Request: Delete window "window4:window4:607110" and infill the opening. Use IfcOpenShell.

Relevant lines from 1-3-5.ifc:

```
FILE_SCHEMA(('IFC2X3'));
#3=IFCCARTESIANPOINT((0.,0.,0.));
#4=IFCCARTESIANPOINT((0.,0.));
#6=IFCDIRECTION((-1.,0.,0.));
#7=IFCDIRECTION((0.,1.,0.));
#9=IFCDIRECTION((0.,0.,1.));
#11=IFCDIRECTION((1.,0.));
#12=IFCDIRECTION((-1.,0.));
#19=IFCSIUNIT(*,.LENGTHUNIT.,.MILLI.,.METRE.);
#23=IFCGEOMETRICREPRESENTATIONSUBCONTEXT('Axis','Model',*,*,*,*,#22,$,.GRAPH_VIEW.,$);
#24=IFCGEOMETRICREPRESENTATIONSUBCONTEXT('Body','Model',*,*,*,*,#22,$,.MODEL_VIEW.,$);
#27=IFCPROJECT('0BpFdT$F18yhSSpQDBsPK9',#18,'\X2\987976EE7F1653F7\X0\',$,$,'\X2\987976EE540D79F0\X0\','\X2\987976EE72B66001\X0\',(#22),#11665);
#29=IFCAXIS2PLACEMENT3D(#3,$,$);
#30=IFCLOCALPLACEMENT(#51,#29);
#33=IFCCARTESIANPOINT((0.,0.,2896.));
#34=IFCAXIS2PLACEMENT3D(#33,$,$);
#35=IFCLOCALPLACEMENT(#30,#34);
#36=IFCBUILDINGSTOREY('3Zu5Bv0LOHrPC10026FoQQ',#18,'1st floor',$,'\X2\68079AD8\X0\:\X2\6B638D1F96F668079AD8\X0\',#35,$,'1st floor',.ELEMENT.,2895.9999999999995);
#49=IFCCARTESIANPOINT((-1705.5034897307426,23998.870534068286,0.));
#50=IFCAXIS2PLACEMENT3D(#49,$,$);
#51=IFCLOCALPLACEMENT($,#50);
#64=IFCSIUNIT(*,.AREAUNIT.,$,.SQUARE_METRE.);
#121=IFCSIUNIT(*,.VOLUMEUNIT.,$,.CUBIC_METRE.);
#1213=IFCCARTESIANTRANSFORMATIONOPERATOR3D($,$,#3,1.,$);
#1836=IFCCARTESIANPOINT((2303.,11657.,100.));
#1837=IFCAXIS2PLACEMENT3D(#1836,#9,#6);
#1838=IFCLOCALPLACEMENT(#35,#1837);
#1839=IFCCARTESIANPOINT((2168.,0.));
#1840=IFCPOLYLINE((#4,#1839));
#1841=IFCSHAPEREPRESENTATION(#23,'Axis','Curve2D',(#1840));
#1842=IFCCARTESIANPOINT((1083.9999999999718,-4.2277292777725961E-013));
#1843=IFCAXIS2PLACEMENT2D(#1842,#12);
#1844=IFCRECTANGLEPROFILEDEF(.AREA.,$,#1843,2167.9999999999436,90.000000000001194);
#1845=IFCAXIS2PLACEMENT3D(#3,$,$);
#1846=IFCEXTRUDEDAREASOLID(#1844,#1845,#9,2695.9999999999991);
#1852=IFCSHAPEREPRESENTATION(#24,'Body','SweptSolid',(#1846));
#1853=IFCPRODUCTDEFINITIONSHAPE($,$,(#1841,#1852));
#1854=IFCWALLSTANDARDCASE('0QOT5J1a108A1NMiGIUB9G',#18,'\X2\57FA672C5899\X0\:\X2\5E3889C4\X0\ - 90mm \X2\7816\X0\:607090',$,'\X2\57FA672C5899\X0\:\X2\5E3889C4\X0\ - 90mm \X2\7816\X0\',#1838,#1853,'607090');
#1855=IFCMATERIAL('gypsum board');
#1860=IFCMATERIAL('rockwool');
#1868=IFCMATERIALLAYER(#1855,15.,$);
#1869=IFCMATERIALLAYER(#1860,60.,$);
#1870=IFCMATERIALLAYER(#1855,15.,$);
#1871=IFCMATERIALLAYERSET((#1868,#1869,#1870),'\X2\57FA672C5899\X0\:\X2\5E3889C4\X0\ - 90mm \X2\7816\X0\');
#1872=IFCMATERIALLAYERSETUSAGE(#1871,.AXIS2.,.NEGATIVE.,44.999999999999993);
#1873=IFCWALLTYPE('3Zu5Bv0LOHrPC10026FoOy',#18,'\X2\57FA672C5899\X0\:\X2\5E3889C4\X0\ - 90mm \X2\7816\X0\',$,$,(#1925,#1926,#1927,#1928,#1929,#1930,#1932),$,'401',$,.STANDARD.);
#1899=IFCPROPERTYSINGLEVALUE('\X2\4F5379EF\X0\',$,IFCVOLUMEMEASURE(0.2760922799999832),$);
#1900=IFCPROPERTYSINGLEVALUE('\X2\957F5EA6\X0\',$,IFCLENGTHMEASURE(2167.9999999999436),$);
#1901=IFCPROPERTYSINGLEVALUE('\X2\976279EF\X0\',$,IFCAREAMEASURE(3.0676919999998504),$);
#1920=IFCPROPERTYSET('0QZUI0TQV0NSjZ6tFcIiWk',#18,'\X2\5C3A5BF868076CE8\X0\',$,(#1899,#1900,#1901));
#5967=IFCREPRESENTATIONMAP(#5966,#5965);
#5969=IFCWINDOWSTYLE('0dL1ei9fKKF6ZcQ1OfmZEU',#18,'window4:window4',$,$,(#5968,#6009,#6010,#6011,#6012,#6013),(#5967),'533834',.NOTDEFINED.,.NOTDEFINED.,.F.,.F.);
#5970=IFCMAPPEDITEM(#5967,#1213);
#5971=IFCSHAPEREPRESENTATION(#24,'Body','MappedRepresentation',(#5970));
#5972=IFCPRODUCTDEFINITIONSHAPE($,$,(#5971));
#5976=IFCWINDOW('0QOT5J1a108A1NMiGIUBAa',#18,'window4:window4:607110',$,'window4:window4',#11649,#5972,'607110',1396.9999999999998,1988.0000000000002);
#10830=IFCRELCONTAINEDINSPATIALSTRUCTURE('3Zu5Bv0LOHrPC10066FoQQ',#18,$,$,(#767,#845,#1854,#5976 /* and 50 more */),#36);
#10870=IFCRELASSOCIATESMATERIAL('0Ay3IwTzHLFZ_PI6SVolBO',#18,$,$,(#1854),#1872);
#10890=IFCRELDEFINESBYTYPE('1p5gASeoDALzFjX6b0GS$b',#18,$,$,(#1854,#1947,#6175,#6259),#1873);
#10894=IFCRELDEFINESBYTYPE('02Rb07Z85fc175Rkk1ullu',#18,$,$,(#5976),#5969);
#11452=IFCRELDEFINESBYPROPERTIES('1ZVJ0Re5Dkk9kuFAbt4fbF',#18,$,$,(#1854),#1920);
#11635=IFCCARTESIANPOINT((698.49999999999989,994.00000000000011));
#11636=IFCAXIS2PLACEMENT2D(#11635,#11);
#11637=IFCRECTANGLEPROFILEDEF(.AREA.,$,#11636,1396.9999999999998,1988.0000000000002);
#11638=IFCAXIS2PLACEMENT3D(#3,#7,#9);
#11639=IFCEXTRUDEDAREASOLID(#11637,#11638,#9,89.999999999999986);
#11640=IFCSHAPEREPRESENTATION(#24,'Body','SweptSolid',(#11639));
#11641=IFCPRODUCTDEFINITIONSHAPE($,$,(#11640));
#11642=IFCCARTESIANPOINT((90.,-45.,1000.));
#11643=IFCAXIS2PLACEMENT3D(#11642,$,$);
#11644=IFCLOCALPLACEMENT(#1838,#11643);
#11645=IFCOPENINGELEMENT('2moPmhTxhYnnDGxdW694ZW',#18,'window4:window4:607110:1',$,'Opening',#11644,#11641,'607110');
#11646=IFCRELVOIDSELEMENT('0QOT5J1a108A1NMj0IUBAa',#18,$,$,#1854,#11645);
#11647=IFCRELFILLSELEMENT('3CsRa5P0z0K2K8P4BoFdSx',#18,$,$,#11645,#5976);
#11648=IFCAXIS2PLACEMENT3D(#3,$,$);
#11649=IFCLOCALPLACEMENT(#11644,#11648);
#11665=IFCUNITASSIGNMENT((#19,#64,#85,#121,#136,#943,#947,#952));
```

```python
import ifcopenshell
import ifcopenshell.api.feature
import ifcopenshell.api.pset
import ifcopenshell.api.root
import ifcopenshell.geom
import ifcopenshell.util.element
import ifcopenshell.util.shape
import ifcopenshell.util.unit

model = ifcopenshell.open("1-3-5.ifc")
area_scale = ifcopenshell.util.unit.calculate_unit_scale(model, "AREAUNIT")
volume_scale = ifcopenshell.util.unit.calculate_unit_scale(model, "VOLUMEUNIT")
settings = ifcopenshell.geom.settings()


def volume(element):
    """Net volume in cubic metres, openings subtracted."""
    shape = ifcopenshell.geom.create_shape(settings, element)
    return ifcopenshell.util.shape.get_volume(shape.geometry)


window = model.by_id(5976)
opening = window.FillsVoids[0].RelatingOpeningElement
wall = opening.VoidsElements[0].RelatingBuildingElement
before = volume(wall)

ifcopenshell.api.root.remove_product(model, product=window)
ifcopenshell.api.feature.remove_feature(model, feature=opening)

after = volume(wall)
thickness = 0.09  # wall thickness in metres

# Update the wall's stored quantities.
pset = model.by_id(ifcopenshell.util.element.get_pset(wall, "尺寸标注", should_inherit=False)["id"])
ifcopenshell.api.pset.edit_pset(model, pset=pset, properties={
    "体积": model.create_entity("IfcVolumeMeasure", after / volume_scale),
    "面积": model.create_entity("IfcAreaMeasure", after / thickness / area_scale),
})

print(f"wall volume {before:.3f} -> {after:.3f} m3")

model.write("1-3-5_edited.ifc")
```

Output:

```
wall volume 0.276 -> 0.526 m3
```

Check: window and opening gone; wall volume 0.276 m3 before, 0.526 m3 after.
